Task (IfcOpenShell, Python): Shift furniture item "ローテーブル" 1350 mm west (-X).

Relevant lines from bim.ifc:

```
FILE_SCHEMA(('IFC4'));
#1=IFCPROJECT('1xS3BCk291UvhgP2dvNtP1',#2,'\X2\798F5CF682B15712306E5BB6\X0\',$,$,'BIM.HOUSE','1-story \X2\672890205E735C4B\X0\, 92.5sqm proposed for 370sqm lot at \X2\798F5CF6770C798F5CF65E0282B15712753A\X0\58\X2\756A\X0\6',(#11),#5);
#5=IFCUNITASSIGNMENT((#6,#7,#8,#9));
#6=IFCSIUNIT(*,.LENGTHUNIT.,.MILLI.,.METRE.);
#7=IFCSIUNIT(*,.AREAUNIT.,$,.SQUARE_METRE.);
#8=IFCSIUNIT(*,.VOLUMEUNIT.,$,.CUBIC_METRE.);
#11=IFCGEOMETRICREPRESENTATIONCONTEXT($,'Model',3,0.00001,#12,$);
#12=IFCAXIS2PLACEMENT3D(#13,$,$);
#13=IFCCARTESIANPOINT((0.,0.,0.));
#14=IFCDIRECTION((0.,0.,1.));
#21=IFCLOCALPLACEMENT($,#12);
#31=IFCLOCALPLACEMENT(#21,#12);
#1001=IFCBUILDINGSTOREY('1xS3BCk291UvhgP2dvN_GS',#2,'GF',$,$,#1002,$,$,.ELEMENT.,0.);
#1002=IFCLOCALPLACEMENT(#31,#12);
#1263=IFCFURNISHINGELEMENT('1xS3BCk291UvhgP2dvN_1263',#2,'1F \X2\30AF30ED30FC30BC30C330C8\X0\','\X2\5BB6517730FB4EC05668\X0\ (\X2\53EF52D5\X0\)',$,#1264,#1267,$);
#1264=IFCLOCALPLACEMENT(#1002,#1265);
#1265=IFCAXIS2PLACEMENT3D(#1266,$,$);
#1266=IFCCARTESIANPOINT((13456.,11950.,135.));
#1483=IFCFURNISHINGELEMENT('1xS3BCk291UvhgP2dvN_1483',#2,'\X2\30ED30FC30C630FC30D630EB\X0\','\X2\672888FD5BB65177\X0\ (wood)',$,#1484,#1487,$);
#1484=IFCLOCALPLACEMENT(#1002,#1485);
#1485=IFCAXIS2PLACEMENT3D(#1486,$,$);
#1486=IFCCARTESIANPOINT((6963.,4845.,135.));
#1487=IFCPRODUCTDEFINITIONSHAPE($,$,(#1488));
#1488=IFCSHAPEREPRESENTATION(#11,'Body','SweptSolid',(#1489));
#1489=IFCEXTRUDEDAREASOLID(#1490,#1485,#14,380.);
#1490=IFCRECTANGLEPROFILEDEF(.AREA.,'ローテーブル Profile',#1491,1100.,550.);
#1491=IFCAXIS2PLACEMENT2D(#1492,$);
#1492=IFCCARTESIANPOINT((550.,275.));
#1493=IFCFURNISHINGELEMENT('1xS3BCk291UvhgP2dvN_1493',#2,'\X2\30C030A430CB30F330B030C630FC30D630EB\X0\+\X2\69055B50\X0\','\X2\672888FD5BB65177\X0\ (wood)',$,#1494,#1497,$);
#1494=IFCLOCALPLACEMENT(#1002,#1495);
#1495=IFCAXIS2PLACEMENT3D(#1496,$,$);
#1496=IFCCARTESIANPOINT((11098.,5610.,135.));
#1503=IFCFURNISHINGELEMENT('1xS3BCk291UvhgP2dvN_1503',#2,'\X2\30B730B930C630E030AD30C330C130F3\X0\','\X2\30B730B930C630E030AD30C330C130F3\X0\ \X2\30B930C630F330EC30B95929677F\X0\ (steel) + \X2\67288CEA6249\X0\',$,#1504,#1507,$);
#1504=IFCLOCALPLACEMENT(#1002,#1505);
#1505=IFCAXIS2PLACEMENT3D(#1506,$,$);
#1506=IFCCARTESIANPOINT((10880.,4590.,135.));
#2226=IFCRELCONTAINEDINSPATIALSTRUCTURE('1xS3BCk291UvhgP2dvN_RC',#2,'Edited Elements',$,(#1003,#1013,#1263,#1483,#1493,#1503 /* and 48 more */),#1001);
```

```python
import ifcopenshell
import ifcopenshell.api.geometry
import ifcopenshell.util.placement
import ifcopenshell.util.unit

model = ifcopenshell.open("bim.ifc")
unit_scale = ifcopenshell.util.unit.calculate_unit_scale(model)

item = model.by_guid("1xS3BCk291UvhgP2dvN_1483")
matrix = ifcopenshell.util.placement.get_local_placement(item.ObjectPlacement)
matrix[0, 3] -= 1.35 / unit_scale
ifcopenshell.api.geometry.edit_object_placement(model, product=item, matrix=matrix, is_si=False)

print(ifcopenshell.util.placement.get_local_placement(item.ObjectPlacement).round(3) + 0.0)

model.write("bim_edited.ifc")
```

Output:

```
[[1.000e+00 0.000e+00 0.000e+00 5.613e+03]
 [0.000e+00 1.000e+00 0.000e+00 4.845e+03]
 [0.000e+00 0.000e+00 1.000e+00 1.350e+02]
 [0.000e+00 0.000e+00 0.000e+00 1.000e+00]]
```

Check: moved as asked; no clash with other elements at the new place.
